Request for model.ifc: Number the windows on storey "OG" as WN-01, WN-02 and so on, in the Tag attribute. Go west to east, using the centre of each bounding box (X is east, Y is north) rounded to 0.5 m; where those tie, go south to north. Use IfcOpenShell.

First a look at what the model holds.

```python
import ifcopenshell
import ifcopenshell.util.element
import ifcopenshell.util.placement

model = ifcopenshell.open("model.ifc")
print(model.schema)
storey = next(s for s in model.by_type("IfcBuildingStorey") if s.Name == "OG")
windows = [e for e in ifcopenshell.util.element.get_decomposition(storey) if e.is_a("IfcWindow")]
for e in sorted(windows, key=lambda e: e.id()):
    origin = ifcopenshell.util.placement.get_local_placement(e.ObjectPlacement)[:3, 3]
    print(e.id(), e.Tag, e.Name, origin.round(2) + 0.0, sep=" | ")
```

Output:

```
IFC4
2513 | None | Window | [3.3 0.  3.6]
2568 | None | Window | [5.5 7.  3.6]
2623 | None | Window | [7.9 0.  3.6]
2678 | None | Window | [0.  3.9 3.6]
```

```python
import ifcopenshell
import ifcopenshell.geom
import ifcopenshell.util.element
import ifcopenshell.util.shape

model = ifcopenshell.open("model.ifc")
settings = ifcopenshell.geom.settings()
settings.set("use-world-coords", True)


def centre(element):
    shape = ifcopenshell.geom.create_shape(settings, element)
    return ifcopenshell.util.shape.get_bbox_centroid(shape.geometry)


storey = next(s for s in model.by_type("IfcBuildingStorey") if s.Name == "OG")
windows = [e for e in ifcopenshell.util.element.get_decomposition(storey) if e.is_a("IfcWindow")]

# Insertion points can sit at a corner or the storey origin, so sort by the geometry (in metres).
centres = {e: centre(e) for e in windows}
windows.sort(key=lambda e: (round(centres[e][0] / 0.5), centres[e][1]))

for i, e in enumerate(windows, start=1):
    number = f"WN-{i:02d}"
    e.Tag = number
    print(e.id(), number)

model.write("model_edited.ifc")
```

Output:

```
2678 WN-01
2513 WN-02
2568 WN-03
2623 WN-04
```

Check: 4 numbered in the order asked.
